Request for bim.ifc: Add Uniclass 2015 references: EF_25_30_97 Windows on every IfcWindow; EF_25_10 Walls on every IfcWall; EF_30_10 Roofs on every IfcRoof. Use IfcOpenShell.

First a look at what the model holds.

```python
import ifcopenshell

model = ifcopenshell.open("bim.ifc")
print(model.schema)
print("classifications:", [c.Name for c in model.by_type("IfcClassification")])
for ifc_class in ("IfcDoor", "IfcRoof", "IfcStair", "IfcWall", "IfcWindow"):
    print(ifc_class, len(model.by_type(ifc_class)))
```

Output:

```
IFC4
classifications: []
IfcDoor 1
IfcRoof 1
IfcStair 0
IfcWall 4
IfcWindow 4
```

```python
import ifcopenshell
import ifcopenshell.api.classification

model = ifcopenshell.open("bim.ifc")

system = ifcopenshell.api.classification.add_classification(model, classification="Uniclass 2015")

codes = {
    "IfcWindow": ("EF_25_30_97", "Windows"),
    "IfcWall": ("EF_25_10", "Walls"),
    "IfcRoof": ("EF_30_10", "Roofs"),
}
for ifc_class, (code, name) in codes.items():
    products = model.by_type(ifc_class)
    ifcopenshell.api.classification.add_reference(
        model, products=products, classification=system, identification=code, name=name
    )
    print(code, len(products))

model.write("bim_rev.ifc")
```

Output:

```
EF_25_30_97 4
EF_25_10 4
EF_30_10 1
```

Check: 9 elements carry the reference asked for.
